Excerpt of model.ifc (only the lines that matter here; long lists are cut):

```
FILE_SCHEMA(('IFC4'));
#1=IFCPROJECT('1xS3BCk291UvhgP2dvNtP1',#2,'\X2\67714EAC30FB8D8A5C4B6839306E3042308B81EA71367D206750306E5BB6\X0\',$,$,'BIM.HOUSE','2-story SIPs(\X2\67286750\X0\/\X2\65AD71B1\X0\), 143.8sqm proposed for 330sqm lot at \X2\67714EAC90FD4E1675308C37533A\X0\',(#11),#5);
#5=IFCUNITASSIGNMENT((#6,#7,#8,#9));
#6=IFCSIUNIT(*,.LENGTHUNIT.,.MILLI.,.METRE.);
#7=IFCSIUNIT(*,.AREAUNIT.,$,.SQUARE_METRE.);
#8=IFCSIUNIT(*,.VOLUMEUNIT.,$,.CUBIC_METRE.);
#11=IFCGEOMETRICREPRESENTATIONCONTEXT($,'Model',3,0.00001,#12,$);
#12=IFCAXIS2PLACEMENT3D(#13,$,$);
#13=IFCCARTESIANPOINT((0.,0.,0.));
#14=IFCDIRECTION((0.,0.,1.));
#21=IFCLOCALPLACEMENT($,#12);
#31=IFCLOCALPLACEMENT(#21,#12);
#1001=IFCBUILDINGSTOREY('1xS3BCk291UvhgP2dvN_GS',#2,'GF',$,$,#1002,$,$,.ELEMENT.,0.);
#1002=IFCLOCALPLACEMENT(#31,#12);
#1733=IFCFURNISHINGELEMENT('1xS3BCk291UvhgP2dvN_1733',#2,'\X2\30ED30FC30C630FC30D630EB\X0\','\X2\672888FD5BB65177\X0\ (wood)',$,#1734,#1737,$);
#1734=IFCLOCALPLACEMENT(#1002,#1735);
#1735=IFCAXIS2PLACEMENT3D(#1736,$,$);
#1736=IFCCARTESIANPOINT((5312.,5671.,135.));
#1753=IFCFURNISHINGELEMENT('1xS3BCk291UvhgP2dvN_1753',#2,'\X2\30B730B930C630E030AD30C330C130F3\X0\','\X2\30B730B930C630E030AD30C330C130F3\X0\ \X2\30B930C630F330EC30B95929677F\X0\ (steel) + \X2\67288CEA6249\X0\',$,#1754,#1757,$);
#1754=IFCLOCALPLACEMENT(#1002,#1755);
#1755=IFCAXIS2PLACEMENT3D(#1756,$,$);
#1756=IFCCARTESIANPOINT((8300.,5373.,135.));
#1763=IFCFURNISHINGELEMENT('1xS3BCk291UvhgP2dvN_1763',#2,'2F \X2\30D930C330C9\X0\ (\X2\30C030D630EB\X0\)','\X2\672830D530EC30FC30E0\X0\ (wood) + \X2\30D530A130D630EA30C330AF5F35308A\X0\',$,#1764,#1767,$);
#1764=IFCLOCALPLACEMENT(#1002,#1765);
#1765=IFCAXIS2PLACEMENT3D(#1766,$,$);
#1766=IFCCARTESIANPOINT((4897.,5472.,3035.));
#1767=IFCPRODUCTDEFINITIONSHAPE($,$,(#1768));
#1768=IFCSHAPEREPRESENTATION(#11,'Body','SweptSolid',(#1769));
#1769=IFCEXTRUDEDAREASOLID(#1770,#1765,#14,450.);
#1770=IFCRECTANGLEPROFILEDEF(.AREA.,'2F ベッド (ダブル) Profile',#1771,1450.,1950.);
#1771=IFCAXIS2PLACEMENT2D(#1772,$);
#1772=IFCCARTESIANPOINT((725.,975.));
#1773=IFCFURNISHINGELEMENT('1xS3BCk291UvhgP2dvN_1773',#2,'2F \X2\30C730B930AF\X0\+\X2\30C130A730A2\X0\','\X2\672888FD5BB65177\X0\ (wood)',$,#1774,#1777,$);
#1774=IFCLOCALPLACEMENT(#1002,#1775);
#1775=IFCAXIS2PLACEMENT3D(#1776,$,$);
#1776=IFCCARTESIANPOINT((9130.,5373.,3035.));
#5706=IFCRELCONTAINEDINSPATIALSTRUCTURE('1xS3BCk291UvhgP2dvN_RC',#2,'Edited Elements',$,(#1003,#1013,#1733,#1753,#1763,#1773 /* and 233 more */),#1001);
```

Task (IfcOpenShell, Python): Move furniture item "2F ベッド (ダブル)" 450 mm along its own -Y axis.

```python
import ifcopenshell
import ifcopenshell.api.geometry
import ifcopenshell.util.placement

model = ifcopenshell.open("model.ifc")

item = model.by_guid("1xS3BCk291UvhgP2dvN_1763")
matrix = ifcopenshell.util.placement.get_local_placement(item.ObjectPlacement)
matrix[:3, 3] -= matrix[:3, 1] * 450.0
ifcopenshell.api.geometry.edit_object_placement(model, product=item, matrix=matrix, is_si=False)

print(ifcopenshell.util.placement.get_local_placement(item.ObjectPlacement).round(3) + 0.0)

model.write("model_v2.ifc")
```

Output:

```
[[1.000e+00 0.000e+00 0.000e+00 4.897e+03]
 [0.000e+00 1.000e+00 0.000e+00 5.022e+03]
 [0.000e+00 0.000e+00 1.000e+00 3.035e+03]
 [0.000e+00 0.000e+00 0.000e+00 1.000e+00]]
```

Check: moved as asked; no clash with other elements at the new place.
